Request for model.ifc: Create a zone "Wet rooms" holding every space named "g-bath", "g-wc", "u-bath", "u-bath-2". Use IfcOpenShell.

First a look at what the model holds.

```python
import ifcopenshell

model = ifcopenshell.open("model.ifc")
print(model.schema)
seen = {}
for space in model.by_type("IfcSpace"):
    seen[space.LongName] = seen.get(space.LongName, 0) + 1
for name, count in sorted(seen.items(), key=str):
    print(count, "x", name)
print("zones:", [z.Name for z in model.by_type("IfcZone")][:20])
```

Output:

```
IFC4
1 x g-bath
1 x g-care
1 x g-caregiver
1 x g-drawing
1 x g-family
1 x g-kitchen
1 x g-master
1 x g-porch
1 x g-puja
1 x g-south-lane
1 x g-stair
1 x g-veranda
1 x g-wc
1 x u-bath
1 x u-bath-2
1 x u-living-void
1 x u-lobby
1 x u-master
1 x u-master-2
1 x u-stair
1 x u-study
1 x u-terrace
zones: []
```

```python
import ifcopenshell
import ifcopenshell.api.group
import ifcopenshell.api.root

model = ifcopenshell.open("model.ifc")

names = {"g-bath", "g-wc", "u-bath", "u-bath-2"}
spaces = [s for s in model.by_type("IfcSpace") if s.LongName in names]

zone = ifcopenshell.api.root.create_entity(model, ifc_class="IfcZone", name="Wet rooms")
ifcopenshell.api.group.assign_group(model, products=spaces, group=zone)
print(len(spaces), "spaces in", zone.Name)

model.write("model_updated.ifc")
```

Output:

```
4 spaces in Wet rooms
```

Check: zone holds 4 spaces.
